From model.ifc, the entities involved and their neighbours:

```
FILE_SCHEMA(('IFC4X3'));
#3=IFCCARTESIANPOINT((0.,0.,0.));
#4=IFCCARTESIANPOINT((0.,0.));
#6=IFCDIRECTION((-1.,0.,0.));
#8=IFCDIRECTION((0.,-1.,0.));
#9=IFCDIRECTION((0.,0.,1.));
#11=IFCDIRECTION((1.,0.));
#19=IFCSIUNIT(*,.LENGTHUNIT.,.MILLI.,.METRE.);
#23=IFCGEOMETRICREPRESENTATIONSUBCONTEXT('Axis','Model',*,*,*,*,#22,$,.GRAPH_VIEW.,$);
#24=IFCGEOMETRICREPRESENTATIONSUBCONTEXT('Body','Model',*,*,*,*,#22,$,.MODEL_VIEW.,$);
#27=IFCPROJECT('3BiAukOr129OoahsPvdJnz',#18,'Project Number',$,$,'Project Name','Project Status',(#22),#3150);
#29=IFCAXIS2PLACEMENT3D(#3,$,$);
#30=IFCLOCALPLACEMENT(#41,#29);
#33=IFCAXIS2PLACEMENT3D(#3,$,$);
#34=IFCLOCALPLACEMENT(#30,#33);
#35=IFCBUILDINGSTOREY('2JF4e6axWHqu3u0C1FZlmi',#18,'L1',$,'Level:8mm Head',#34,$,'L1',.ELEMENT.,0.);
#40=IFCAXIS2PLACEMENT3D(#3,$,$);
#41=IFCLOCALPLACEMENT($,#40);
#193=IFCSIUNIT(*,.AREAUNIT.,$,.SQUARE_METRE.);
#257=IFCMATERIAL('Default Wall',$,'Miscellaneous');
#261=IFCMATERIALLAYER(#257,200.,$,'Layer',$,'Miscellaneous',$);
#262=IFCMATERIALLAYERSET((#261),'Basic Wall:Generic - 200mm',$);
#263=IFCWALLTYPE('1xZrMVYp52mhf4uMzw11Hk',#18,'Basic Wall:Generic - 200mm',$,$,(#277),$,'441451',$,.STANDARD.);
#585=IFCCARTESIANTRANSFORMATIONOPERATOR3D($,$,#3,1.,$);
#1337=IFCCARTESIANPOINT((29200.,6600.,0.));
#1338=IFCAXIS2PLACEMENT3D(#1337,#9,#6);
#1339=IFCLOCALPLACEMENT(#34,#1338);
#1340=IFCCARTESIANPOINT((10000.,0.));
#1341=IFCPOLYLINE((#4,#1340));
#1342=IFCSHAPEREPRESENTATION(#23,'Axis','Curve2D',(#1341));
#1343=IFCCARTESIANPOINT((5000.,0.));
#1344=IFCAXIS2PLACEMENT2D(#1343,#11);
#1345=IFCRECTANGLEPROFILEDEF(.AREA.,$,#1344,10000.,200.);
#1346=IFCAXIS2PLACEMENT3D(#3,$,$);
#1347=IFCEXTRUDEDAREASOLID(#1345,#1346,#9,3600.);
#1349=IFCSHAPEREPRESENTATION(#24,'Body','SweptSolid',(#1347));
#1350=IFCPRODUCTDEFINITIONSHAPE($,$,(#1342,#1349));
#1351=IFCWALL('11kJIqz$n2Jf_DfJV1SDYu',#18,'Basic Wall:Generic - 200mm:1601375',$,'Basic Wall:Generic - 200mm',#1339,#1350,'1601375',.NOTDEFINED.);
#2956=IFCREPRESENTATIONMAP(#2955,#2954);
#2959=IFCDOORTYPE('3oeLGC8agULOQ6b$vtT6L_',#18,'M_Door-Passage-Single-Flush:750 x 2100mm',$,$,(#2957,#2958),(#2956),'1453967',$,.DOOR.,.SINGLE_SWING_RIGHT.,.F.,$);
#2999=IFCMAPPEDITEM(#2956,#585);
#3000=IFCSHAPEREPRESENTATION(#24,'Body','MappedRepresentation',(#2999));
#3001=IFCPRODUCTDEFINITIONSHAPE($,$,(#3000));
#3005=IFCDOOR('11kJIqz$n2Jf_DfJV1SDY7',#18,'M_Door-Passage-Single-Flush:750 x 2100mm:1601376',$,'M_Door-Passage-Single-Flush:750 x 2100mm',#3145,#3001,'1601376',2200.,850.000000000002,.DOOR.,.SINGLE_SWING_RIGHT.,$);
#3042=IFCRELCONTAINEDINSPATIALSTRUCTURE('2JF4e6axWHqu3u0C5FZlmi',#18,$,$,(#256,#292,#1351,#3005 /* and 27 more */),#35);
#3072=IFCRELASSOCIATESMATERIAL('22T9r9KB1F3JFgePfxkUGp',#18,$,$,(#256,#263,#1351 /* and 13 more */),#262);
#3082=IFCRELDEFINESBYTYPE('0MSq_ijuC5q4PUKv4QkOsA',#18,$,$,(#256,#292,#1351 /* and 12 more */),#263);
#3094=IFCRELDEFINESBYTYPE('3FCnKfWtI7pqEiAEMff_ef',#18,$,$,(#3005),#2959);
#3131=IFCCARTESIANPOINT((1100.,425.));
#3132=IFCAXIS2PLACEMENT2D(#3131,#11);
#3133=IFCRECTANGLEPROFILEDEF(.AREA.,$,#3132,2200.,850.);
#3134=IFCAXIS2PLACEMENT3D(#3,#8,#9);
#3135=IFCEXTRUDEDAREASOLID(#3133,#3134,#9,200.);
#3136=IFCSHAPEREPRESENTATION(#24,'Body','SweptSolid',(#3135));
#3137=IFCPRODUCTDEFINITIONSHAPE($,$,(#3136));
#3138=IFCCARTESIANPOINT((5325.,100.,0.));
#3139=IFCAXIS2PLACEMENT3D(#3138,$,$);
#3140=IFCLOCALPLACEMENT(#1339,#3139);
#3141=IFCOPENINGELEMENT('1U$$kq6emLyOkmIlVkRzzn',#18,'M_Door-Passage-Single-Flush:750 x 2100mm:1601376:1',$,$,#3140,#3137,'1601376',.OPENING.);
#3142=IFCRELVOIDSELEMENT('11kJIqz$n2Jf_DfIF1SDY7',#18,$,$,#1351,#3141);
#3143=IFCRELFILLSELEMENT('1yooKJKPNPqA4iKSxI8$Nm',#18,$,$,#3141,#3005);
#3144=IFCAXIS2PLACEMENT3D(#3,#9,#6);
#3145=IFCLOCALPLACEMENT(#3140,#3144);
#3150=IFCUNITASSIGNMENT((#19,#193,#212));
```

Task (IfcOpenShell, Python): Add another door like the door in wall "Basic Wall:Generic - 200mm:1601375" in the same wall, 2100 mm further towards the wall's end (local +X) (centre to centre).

```python
import ifcopenshell
import ifcopenshell.api.feature
import ifcopenshell.api.geometry
import ifcopenshell.api.root
import ifcopenshell.geom
import ifcopenshell.util.element
import ifcopenshell.util.placement
import ifcopenshell.util.shape
import ifcopenshell.util.unit

model = ifcopenshell.open("model.ifc")
unit_scale = ifcopenshell.util.unit.calculate_unit_scale(model)
settings = ifcopenshell.geom.settings()


def volume(element):
    """Net volume in cubic metres, openings subtracted."""
    shape = ifcopenshell.geom.create_shape(settings, element)
    return ifcopenshell.util.shape.get_volume(shape.geometry)


def reuse_history(source, copy):
    """copy_class also copies each property set's owner history, people and application; keep the originals."""
    for rel in copy.IsDefinedBy:
        if rel.is_a("IfcRelDefinesByProperties") and (history := rel.RelatingPropertyDefinition.OwnerHistory):
            rel.RelatingPropertyDefinition.OwnerHistory = source.OwnerHistory
            ifcopenshell.util.element.remove_deep2(model, history)


door = model.by_id(3005)
opening = door.FillsVoids[0].RelatingOpeningElement
wall = opening.VoidsElements[0].RelatingBuildingElement
before = volume(wall)
shift = ifcopenshell.util.placement.get_local_placement(wall.ObjectPlacement)[:3, 0] * 2.1 / unit_scale

# copy_class copies the void relationship, type, container and properties, but no geometry.
new_opening = ifcopenshell.api.root.copy_class(model, product=opening)
new_opening.Representation = ifcopenshell.util.element.copy_deep(
    model, opening.Representation, exclude=["IfcGeometricRepresentationContext", "IfcRepresentationMap"]
)
new_opening.Name = "M_Door-Passage-Single-Flush:750 x 2100mm"
new_opening.Tag = None
new_door = ifcopenshell.api.root.copy_class(model, product=door)
new_door.Representation = ifcopenshell.util.element.copy_deep(
    model, door.Representation, exclude=["IfcGeometricRepresentationContext", "IfcRepresentationMap"]
)
new_door.Name = "M_Door-Passage-Single-Flush:750 x 2100mm"
new_door.Tag = None
reuse_history(door, new_door)
ifcopenshell.api.feature.add_filling(model, opening=new_opening, element=new_door)

for old, new in ((opening, new_opening), (door, new_door)):
    matrix = ifcopenshell.util.placement.get_local_placement(old.ObjectPlacement)
    matrix[:3, 3] += shift
    ifcopenshell.api.geometry.edit_object_placement(model, product=new, matrix=matrix, is_si=False)

after = volume(wall)

print(f"wall volume {before:.3f} -> {after:.3f} m3")

model.write("model_edited.ifc")
```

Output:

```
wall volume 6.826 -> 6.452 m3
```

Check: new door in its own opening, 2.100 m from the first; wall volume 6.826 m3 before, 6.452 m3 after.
